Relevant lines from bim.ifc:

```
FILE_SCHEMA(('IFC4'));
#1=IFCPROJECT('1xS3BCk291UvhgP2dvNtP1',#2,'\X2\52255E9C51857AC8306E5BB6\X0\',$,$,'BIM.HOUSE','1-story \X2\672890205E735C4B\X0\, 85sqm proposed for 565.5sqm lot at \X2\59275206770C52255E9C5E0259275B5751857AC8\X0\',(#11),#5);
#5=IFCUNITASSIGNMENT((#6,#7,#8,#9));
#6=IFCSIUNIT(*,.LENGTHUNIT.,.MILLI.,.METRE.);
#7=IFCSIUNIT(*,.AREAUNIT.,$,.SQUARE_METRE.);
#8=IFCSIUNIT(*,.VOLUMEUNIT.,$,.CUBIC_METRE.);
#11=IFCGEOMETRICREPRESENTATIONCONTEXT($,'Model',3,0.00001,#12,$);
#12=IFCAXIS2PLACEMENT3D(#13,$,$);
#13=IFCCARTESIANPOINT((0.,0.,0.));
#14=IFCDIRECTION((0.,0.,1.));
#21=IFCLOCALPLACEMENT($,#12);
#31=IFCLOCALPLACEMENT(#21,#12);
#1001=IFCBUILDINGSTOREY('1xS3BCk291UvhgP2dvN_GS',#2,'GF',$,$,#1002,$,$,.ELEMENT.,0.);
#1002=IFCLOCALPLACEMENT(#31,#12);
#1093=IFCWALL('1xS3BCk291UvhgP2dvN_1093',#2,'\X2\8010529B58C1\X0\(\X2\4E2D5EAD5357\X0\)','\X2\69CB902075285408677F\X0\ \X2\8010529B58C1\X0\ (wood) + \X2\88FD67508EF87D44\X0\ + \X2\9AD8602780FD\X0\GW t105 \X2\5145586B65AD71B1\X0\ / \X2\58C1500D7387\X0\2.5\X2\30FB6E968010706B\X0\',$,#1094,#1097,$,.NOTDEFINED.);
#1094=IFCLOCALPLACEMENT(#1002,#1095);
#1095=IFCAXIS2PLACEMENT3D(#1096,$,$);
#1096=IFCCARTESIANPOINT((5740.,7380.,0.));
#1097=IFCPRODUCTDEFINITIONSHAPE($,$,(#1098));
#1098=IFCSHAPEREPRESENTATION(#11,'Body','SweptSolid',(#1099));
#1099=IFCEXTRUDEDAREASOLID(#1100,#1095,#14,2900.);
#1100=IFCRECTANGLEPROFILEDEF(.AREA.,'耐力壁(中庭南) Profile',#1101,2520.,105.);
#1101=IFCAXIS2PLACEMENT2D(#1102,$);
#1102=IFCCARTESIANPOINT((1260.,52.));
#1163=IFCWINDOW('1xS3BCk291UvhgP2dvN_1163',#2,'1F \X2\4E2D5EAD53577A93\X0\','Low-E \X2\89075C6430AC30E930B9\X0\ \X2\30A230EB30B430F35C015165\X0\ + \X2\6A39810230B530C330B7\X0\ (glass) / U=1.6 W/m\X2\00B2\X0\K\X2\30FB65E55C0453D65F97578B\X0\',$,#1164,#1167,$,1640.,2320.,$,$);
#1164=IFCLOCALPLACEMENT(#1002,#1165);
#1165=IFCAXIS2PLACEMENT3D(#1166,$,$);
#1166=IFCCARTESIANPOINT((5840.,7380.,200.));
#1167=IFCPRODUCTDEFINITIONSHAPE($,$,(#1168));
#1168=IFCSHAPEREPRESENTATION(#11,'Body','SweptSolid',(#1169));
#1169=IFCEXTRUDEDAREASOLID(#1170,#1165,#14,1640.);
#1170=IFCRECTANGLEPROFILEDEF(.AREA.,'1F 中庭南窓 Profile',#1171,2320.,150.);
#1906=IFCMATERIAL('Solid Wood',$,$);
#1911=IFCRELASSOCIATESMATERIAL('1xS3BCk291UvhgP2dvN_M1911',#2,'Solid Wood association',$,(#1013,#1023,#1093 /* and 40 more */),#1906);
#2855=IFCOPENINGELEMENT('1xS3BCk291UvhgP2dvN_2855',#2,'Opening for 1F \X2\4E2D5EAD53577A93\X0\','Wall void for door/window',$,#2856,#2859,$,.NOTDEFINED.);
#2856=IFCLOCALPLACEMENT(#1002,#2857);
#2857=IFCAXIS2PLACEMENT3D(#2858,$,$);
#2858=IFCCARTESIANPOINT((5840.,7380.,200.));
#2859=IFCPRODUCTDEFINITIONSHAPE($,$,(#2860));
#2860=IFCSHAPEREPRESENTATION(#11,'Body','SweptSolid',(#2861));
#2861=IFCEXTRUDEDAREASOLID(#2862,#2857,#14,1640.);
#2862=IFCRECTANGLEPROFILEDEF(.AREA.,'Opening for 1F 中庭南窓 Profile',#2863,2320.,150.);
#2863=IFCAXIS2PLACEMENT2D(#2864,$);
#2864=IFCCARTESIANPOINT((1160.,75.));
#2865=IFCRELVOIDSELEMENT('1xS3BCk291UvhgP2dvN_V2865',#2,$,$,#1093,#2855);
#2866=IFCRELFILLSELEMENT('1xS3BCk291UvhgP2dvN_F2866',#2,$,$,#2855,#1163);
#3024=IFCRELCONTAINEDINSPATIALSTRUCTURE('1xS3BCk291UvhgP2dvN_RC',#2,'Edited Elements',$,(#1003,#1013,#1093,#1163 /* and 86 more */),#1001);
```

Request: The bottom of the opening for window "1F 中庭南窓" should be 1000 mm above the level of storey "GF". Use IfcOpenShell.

```python
import numpy as np
import ifcopenshell
import ifcopenshell.api.geometry
import ifcopenshell.geom
import ifcopenshell.util.element
import ifcopenshell.util.placement
import ifcopenshell.util.shape
import ifcopenshell.util.unit

model = ifcopenshell.open("bim.ifc")
unit_scale = ifcopenshell.util.unit.calculate_unit_scale(model)

window = model.by_guid("1xS3BCk291UvhgP2dvN_1163")
opening = window.FillsVoids[0].RelatingOpeningElement
storey = ifcopenshell.util.element.get_container(window, ifc_class="IfcBuildingStorey")
level = ifcopenshell.util.placement.get_local_placement(storey.ObjectPlacement)[2, 3]

# The opening's origin need not be at the sill, so measure its lowest point.
shape = ifcopenshell.geom.create_shape(ifcopenshell.geom.settings(), opening)
bottom = ifcopenshell.util.shape.get_shape_bottom_elevation(shape, shape.geometry) / unit_scale
dz = level + 1 / unit_scale - bottom

shift = np.array([0.0, 0.0, dz])
# The window is not placed relative to its opening, so move both.
for product in (opening, window):
    matrix = ifcopenshell.util.placement.get_local_placement(product.ObjectPlacement)
    matrix[:3, 3] += shift
    ifcopenshell.api.geometry.edit_object_placement(model, product=product, matrix=matrix, is_si=False)

print(f"moved by {dz * unit_scale:+.3f} m")

model.write("bim_rev.ifc")
```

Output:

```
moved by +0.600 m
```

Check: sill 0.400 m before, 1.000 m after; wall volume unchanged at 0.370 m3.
